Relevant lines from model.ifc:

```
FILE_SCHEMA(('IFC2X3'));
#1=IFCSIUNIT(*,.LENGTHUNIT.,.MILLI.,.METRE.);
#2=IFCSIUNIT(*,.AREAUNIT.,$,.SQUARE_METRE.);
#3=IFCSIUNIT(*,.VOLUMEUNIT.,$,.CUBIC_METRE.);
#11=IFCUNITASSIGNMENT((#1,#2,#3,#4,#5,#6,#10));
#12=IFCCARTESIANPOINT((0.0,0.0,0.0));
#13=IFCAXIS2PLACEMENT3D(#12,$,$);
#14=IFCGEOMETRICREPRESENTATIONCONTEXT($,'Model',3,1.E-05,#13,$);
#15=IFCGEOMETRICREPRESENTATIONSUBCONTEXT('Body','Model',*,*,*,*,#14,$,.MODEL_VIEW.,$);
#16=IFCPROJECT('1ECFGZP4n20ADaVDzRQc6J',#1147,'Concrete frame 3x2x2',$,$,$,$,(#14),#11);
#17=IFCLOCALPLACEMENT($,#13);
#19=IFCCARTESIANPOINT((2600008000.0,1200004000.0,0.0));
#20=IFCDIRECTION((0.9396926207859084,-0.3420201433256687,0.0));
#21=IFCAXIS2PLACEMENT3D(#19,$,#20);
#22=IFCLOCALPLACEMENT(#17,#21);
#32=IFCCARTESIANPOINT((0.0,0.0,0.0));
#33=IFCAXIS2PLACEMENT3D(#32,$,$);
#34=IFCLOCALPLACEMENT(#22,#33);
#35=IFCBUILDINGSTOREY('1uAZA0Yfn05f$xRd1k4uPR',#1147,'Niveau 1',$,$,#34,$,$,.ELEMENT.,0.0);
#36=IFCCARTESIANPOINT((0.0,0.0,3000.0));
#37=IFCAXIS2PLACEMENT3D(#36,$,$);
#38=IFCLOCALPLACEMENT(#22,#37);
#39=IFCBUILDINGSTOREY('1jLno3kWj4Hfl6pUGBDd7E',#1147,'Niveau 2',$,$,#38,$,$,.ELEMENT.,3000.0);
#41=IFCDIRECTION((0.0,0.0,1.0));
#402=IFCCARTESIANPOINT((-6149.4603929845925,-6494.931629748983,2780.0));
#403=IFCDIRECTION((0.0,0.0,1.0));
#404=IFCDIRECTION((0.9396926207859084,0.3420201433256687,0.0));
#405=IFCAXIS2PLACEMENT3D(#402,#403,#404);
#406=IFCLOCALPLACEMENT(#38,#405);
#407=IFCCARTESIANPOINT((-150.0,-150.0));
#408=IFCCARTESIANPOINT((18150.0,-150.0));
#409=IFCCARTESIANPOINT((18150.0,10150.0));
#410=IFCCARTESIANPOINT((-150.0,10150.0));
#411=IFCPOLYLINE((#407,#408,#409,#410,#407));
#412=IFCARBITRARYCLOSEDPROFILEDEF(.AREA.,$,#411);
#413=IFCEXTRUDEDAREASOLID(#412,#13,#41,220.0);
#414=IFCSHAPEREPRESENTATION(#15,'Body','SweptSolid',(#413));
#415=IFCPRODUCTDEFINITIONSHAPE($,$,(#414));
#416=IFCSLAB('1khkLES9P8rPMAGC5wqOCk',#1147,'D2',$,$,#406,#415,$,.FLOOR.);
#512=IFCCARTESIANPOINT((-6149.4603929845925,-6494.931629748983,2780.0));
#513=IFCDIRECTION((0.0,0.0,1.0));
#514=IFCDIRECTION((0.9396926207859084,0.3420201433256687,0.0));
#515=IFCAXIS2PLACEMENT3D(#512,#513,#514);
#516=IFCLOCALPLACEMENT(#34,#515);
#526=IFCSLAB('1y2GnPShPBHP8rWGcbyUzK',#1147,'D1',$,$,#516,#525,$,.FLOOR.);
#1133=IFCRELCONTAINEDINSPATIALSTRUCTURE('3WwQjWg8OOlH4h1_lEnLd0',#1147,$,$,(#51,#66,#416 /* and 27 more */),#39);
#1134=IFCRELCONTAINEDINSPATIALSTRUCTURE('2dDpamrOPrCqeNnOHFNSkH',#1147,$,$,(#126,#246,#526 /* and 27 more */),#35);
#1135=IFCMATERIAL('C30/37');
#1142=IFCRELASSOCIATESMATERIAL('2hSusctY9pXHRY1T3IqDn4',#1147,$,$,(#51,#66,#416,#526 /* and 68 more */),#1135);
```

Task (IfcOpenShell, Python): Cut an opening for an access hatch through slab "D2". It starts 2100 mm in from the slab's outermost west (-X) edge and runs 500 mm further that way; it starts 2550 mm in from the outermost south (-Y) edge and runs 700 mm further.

```python
import numpy as np
import ifcopenshell
import ifcopenshell.api.feature
import ifcopenshell.api.geometry
import ifcopenshell.api.root
import ifcopenshell.geom
import ifcopenshell.util.placement
import ifcopenshell.util.representation
import ifcopenshell.util.shape
import ifcopenshell.util.unit

model = ifcopenshell.open("model.ifc")
unit_scale = ifcopenshell.util.unit.calculate_unit_scale(model)
settings = ifcopenshell.geom.settings()


def volume(element):
    """Net volume in cubic metres, openings subtracted."""
    shape = ifcopenshell.geom.create_shape(settings, element)
    return ifcopenshell.util.shape.get_volume(shape.geometry)


slab = model.by_id(416)
before = volume(slab)

# Extent in the slab's own axes, in metres. The edges named are its -X and -Y sides.
slab_shape = ifcopenshell.geom.create_shape(settings, slab)
vertices = ifcopenshell.util.shape.get_vertices(slab_shape.geometry)
x_min, y_min, bottom = vertices.min(axis=0)
top = vertices[:, 2].max()

opening = ifcopenshell.api.root.create_entity(model, ifc_class="IfcOpeningElement", name="Access hatch opening")
context = ifcopenshell.util.representation.get_context(model, "Model", "Body", "MODEL_VIEW")
width, depth = 0.5, 0.7
outline = [(0.0, 0.0), (width, 0.0), (width, depth), (0.0, depth), (0.0, 0.0)]
# Overshoot both faces by 50 mm so the cut is clean.
shape = ifcopenshell.api.geometry.add_slab_representation(
    model, context=context, depth=top - bottom + 0.1, polyline=outline
)
ifcopenshell.api.geometry.assign_representation(model, product=opening, representation=shape)

matrix = ifcopenshell.util.placement.get_local_placement(slab.ObjectPlacement)
matrix[:, 3] = matrix @ np.append(np.array([x_min + 2.1, y_min + 2.55, bottom - 0.05]) / unit_scale, 1.0)
ifcopenshell.api.geometry.edit_object_placement(model, product=opening, matrix=matrix, is_si=False)
ifcopenshell.api.feature.add_feature(model, feature=opening, element=slab)

after = volume(slab)

print(f"slab volume {before:.3f} -> {after:.3f} m3")

model.write("model-out.ifc")
```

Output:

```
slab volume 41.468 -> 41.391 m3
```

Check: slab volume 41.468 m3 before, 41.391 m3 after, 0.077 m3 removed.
